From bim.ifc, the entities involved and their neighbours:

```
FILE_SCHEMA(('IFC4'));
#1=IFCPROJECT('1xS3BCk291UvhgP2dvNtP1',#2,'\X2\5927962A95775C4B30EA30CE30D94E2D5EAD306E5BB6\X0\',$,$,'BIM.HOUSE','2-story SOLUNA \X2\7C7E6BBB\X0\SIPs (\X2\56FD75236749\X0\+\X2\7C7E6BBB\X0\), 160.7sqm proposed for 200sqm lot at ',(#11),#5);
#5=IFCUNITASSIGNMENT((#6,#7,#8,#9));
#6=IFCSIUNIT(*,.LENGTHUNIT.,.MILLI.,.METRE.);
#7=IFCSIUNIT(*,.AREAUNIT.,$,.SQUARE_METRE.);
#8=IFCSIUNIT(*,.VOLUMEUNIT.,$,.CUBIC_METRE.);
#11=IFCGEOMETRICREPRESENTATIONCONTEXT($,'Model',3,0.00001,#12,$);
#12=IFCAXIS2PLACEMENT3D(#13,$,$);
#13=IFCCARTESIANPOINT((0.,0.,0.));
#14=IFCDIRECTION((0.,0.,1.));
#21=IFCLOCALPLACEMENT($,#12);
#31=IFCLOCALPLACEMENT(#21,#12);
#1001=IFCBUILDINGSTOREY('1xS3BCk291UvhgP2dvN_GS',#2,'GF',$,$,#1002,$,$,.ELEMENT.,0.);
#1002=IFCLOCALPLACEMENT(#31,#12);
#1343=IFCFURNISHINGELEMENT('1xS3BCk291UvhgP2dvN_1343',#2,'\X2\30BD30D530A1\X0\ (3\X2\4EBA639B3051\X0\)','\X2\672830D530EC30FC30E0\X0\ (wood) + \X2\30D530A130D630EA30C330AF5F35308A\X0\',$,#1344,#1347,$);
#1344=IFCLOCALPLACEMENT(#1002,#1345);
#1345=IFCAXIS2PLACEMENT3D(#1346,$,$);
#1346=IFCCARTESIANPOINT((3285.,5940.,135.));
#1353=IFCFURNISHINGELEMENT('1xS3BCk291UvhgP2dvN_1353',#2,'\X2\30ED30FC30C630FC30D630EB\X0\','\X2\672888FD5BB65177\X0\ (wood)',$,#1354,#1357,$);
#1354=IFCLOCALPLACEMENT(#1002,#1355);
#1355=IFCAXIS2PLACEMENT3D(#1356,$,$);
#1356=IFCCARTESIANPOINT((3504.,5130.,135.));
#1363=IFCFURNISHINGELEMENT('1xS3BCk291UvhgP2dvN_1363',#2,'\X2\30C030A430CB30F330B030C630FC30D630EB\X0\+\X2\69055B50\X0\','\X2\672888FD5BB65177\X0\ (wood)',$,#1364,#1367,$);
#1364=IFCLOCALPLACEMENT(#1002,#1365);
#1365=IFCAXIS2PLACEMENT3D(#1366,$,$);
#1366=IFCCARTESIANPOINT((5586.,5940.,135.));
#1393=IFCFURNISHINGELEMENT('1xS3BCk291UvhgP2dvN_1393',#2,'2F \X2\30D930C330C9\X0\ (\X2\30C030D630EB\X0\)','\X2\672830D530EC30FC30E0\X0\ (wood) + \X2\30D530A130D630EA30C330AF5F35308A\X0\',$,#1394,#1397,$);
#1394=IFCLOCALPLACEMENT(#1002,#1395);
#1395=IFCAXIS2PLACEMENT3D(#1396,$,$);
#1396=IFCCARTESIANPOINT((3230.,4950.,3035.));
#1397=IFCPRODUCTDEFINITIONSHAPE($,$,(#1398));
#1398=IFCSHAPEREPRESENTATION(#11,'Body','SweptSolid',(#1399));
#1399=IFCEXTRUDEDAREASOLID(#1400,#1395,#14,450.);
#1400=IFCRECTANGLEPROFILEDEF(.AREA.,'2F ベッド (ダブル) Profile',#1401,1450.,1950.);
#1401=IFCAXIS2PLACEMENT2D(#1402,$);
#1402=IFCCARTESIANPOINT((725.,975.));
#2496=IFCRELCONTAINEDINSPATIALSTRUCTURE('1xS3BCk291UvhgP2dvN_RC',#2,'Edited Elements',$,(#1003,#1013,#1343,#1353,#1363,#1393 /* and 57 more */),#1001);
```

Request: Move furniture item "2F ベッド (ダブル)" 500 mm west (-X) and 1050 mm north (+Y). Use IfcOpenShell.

```python
import ifcopenshell
import ifcopenshell.api.geometry
import ifcopenshell.util.placement
import ifcopenshell.util.unit

model = ifcopenshell.open("bim.ifc")
unit_scale = ifcopenshell.util.unit.calculate_unit_scale(model)

item = model.by_guid("1xS3BCk291UvhgP2dvN_1393")
matrix = ifcopenshell.util.placement.get_local_placement(item.ObjectPlacement)
matrix[0, 3] -= 0.5 / unit_scale
matrix[1, 3] += 1.05 / unit_scale
ifcopenshell.api.geometry.edit_object_placement(model, product=item, matrix=matrix, is_si=False)

print(ifcopenshell.util.placement.get_local_placement(item.ObjectPlacement).round(3) + 0.0)

model.write("bim_rev.ifc")
```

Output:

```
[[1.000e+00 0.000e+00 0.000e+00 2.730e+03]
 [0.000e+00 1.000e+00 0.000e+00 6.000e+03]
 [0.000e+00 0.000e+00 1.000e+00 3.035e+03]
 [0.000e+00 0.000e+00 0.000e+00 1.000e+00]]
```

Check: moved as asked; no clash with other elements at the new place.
